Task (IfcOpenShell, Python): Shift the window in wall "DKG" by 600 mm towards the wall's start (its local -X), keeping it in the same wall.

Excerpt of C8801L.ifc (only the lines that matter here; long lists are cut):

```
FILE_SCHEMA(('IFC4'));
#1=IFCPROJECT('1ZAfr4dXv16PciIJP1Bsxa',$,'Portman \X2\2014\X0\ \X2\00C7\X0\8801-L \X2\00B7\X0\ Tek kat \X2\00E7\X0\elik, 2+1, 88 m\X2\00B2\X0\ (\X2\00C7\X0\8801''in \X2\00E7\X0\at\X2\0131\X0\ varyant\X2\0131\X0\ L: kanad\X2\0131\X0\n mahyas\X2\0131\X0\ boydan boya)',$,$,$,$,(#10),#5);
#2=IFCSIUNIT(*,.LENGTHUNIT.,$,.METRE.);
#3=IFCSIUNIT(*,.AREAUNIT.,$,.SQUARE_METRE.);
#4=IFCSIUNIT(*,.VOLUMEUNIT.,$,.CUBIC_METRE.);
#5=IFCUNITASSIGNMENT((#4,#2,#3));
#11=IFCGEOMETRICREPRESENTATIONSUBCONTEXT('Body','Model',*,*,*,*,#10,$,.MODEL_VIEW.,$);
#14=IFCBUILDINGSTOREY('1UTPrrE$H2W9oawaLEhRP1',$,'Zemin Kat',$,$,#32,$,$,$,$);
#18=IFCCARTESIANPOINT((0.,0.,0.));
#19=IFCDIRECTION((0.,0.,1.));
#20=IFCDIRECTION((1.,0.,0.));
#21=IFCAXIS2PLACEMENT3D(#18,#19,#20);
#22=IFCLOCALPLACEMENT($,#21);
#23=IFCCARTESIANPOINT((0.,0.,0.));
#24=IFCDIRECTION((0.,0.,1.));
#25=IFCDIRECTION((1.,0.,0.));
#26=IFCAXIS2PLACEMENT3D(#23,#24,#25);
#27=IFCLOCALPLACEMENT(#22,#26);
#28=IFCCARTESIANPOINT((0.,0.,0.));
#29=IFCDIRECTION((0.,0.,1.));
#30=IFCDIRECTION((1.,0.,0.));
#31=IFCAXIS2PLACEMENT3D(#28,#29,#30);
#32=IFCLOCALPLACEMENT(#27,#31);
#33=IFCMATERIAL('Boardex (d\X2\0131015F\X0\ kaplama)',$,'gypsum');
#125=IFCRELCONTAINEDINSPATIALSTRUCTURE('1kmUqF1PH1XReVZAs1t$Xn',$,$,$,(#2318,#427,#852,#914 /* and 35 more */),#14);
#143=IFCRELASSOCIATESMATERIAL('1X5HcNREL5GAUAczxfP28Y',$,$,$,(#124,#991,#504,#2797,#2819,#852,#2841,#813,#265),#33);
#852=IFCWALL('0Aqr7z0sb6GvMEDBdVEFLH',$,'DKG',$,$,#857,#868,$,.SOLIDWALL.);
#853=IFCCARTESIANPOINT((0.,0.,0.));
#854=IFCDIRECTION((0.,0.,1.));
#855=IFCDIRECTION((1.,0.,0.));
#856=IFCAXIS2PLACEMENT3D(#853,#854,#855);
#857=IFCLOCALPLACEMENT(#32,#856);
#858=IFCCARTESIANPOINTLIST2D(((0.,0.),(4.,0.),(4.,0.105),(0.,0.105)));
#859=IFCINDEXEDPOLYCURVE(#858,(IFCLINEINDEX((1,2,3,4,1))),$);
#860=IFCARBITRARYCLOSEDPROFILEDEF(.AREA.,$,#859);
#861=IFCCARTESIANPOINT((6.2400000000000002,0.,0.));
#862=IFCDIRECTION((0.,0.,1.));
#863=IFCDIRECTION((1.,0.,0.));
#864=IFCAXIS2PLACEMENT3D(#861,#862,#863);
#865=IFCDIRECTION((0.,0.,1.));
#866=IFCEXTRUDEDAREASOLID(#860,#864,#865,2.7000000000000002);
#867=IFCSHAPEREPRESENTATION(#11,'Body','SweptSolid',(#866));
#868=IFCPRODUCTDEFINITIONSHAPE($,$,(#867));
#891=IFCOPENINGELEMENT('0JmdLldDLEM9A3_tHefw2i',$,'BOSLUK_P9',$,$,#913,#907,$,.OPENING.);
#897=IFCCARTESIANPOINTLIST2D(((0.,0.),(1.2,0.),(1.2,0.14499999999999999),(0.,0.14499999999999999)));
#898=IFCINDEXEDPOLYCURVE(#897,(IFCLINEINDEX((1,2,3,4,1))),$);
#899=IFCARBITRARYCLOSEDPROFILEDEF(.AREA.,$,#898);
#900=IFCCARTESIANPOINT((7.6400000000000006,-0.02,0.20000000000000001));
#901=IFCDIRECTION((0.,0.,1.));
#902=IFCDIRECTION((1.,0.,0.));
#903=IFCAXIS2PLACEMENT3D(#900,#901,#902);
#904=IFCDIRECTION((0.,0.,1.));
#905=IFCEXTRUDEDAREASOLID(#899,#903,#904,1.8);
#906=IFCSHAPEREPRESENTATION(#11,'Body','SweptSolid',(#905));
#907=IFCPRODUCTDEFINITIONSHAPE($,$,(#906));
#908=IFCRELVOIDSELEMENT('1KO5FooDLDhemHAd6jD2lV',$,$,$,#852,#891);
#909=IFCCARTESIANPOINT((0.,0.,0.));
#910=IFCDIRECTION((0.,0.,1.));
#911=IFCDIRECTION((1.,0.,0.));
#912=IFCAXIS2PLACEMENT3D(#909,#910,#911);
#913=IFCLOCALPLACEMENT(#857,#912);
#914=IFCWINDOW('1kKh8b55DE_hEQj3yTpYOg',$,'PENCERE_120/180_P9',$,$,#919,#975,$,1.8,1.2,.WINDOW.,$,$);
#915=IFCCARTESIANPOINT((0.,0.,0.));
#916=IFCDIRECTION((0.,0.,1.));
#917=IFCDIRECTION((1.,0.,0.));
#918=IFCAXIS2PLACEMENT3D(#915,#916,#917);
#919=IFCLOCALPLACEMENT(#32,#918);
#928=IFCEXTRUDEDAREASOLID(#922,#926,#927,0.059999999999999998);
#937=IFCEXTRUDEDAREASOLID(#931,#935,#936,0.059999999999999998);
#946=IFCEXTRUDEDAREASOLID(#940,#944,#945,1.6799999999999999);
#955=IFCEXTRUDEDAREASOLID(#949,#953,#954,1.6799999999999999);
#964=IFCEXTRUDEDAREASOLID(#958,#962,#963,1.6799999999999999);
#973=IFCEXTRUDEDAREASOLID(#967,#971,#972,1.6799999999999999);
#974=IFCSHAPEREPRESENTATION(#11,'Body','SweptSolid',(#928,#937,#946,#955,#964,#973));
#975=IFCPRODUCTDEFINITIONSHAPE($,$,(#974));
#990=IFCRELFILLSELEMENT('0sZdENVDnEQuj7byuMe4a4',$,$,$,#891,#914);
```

```python
import ifcopenshell
import ifcopenshell.api.geometry
import ifcopenshell.util.placement

model = ifcopenshell.open("C8801L.ifc")

window = model.by_id(914)
opening = window.FillsVoids[0].RelatingOpeningElement
wall = opening.VoidsElements[0].RelatingBuildingElement

wall_matrix = ifcopenshell.util.placement.get_local_placement(wall.ObjectPlacement)
shift = wall_matrix[:3, 0] * -0.6
before = ifcopenshell.util.placement.get_local_placement(window.ObjectPlacement)[:3, 3].copy()

# The window is not placed relative to its opening, so move both.
for product in (opening, window):
    matrix = ifcopenshell.util.placement.get_local_placement(product.ObjectPlacement)
    matrix[:3, 3] += shift
    ifcopenshell.api.geometry.edit_object_placement(model, product=product, matrix=matrix, is_si=False)

after = ifcopenshell.util.placement.get_local_placement(window.ObjectPlacement)[:3, 3]
print("window moved by", (after - before).round(3) + 0.0)

model.write("C8801L_edited.ifc")
```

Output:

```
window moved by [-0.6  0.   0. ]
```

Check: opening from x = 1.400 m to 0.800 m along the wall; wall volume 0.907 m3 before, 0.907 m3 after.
